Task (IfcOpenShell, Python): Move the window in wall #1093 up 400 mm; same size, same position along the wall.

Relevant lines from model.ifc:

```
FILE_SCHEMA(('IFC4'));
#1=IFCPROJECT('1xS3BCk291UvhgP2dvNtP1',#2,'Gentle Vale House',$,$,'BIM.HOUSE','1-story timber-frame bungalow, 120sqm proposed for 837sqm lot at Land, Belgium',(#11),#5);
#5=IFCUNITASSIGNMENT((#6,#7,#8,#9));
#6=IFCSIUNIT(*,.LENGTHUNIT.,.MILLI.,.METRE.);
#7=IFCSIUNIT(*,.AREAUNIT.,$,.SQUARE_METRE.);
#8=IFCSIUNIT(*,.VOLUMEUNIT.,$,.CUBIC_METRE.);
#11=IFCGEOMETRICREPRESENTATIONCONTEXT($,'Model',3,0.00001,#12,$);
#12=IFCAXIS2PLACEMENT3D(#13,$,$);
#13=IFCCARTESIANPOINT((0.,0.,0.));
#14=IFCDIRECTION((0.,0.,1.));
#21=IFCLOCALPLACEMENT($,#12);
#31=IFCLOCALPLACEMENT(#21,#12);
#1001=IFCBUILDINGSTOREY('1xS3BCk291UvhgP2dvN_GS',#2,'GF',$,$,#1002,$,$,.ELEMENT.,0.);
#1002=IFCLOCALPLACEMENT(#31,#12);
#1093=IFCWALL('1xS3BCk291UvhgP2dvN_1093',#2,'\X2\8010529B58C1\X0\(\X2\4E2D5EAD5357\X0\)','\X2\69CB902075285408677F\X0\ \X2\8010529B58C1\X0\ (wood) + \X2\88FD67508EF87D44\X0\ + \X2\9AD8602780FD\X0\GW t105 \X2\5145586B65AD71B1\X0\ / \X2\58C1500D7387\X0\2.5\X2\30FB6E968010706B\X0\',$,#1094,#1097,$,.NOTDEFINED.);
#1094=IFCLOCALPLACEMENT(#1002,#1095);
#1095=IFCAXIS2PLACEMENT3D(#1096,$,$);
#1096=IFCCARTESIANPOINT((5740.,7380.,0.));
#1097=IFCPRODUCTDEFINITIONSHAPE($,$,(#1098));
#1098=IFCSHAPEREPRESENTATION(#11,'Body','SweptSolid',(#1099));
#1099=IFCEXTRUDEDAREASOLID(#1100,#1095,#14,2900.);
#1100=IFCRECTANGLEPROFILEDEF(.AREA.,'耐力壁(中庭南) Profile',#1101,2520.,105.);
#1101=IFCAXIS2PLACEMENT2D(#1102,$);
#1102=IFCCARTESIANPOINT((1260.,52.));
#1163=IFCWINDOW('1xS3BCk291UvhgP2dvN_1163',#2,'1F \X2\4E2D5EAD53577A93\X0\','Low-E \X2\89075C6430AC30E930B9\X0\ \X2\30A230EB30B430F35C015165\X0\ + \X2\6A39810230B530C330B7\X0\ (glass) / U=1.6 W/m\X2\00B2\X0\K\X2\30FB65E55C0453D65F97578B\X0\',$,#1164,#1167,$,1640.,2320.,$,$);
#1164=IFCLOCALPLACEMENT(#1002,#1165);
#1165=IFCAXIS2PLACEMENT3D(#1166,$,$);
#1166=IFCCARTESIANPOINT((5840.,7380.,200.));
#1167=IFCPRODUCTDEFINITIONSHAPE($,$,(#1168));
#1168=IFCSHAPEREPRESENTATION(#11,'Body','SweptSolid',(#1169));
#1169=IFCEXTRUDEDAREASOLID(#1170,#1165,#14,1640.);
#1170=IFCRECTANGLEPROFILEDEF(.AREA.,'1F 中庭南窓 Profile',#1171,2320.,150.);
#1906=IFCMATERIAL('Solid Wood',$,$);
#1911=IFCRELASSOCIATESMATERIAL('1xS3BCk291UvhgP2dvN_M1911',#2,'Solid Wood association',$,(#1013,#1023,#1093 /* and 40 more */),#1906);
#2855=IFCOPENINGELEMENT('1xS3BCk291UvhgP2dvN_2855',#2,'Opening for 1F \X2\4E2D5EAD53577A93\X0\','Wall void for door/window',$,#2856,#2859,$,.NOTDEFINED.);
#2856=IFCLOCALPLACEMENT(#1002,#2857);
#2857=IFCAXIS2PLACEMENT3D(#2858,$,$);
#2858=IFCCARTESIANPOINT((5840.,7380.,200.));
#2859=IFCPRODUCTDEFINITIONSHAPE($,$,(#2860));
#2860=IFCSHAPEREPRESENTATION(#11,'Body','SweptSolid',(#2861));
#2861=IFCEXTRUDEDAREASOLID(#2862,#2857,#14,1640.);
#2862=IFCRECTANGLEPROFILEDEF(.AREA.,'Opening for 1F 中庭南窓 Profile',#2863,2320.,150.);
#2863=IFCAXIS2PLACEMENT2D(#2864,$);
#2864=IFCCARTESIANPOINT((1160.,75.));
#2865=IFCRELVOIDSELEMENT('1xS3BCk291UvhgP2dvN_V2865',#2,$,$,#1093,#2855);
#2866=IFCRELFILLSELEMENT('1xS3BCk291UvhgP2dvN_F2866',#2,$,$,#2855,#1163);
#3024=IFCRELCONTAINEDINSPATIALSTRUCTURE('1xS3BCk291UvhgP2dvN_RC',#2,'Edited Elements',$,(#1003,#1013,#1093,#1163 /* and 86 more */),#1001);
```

```python
import numpy as np
import ifcopenshell
import ifcopenshell.api.geometry
import ifcopenshell.util.placement
import ifcopenshell.util.unit

model = ifcopenshell.open("model.ifc")
unit_scale = ifcopenshell.util.unit.calculate_unit_scale(model)

window = model.by_id(1163)
opening = window.FillsVoids[0].RelatingOpeningElement
dz = 0.4 / unit_scale

shift = np.array([0.0, 0.0, dz])
# The window is not placed relative to its opening, so move both.
for product in (opening, window):
    matrix = ifcopenshell.util.placement.get_local_placement(product.ObjectPlacement)
    matrix[:3, 3] += shift
    ifcopenshell.api.geometry.edit_object_placement(model, product=product, matrix=matrix, is_si=False)

print(f"moved by {dz * unit_scale:+.3f} m")

model.write("model-out.ifc")
```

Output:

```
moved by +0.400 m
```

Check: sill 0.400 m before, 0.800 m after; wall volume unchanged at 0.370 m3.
